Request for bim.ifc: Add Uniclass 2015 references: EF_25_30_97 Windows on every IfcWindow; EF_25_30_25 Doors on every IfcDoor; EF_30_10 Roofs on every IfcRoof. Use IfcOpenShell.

First a look at what the model holds.

```python
import ifcopenshell

model = ifcopenshell.open("bim.ifc")
print(model.schema)
print("classifications:", [c.Name for c in model.by_type("IfcClassification")])
for ifc_class in ("IfcDoor", "IfcRoof", "IfcStair", "IfcWall", "IfcWindow"):
    print(ifc_class, len(model.by_type(ifc_class)))
```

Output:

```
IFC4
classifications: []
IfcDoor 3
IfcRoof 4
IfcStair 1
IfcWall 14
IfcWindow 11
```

```python
import ifcopenshell
import ifcopenshell.api.classification

model = ifcopenshell.open("bim.ifc")

system = ifcopenshell.api.classification.add_classification(model, classification="Uniclass 2015")

codes = {
    "IfcWindow": ("EF_25_30_97", "Windows"),
    "IfcDoor": ("EF_25_30_25", "Doors"),
    "IfcRoof": ("EF_30_10", "Roofs"),
}
for ifc_class, (code, name) in codes.items():
    products = model.by_type(ifc_class)
    ifcopenshell.api.classification.add_reference(
        model, products=products, classification=system, identification=code, name=name
    )
    print(code, len(products))

model.write("bim_v2.ifc")
```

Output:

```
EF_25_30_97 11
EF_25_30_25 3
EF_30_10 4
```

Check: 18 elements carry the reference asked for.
